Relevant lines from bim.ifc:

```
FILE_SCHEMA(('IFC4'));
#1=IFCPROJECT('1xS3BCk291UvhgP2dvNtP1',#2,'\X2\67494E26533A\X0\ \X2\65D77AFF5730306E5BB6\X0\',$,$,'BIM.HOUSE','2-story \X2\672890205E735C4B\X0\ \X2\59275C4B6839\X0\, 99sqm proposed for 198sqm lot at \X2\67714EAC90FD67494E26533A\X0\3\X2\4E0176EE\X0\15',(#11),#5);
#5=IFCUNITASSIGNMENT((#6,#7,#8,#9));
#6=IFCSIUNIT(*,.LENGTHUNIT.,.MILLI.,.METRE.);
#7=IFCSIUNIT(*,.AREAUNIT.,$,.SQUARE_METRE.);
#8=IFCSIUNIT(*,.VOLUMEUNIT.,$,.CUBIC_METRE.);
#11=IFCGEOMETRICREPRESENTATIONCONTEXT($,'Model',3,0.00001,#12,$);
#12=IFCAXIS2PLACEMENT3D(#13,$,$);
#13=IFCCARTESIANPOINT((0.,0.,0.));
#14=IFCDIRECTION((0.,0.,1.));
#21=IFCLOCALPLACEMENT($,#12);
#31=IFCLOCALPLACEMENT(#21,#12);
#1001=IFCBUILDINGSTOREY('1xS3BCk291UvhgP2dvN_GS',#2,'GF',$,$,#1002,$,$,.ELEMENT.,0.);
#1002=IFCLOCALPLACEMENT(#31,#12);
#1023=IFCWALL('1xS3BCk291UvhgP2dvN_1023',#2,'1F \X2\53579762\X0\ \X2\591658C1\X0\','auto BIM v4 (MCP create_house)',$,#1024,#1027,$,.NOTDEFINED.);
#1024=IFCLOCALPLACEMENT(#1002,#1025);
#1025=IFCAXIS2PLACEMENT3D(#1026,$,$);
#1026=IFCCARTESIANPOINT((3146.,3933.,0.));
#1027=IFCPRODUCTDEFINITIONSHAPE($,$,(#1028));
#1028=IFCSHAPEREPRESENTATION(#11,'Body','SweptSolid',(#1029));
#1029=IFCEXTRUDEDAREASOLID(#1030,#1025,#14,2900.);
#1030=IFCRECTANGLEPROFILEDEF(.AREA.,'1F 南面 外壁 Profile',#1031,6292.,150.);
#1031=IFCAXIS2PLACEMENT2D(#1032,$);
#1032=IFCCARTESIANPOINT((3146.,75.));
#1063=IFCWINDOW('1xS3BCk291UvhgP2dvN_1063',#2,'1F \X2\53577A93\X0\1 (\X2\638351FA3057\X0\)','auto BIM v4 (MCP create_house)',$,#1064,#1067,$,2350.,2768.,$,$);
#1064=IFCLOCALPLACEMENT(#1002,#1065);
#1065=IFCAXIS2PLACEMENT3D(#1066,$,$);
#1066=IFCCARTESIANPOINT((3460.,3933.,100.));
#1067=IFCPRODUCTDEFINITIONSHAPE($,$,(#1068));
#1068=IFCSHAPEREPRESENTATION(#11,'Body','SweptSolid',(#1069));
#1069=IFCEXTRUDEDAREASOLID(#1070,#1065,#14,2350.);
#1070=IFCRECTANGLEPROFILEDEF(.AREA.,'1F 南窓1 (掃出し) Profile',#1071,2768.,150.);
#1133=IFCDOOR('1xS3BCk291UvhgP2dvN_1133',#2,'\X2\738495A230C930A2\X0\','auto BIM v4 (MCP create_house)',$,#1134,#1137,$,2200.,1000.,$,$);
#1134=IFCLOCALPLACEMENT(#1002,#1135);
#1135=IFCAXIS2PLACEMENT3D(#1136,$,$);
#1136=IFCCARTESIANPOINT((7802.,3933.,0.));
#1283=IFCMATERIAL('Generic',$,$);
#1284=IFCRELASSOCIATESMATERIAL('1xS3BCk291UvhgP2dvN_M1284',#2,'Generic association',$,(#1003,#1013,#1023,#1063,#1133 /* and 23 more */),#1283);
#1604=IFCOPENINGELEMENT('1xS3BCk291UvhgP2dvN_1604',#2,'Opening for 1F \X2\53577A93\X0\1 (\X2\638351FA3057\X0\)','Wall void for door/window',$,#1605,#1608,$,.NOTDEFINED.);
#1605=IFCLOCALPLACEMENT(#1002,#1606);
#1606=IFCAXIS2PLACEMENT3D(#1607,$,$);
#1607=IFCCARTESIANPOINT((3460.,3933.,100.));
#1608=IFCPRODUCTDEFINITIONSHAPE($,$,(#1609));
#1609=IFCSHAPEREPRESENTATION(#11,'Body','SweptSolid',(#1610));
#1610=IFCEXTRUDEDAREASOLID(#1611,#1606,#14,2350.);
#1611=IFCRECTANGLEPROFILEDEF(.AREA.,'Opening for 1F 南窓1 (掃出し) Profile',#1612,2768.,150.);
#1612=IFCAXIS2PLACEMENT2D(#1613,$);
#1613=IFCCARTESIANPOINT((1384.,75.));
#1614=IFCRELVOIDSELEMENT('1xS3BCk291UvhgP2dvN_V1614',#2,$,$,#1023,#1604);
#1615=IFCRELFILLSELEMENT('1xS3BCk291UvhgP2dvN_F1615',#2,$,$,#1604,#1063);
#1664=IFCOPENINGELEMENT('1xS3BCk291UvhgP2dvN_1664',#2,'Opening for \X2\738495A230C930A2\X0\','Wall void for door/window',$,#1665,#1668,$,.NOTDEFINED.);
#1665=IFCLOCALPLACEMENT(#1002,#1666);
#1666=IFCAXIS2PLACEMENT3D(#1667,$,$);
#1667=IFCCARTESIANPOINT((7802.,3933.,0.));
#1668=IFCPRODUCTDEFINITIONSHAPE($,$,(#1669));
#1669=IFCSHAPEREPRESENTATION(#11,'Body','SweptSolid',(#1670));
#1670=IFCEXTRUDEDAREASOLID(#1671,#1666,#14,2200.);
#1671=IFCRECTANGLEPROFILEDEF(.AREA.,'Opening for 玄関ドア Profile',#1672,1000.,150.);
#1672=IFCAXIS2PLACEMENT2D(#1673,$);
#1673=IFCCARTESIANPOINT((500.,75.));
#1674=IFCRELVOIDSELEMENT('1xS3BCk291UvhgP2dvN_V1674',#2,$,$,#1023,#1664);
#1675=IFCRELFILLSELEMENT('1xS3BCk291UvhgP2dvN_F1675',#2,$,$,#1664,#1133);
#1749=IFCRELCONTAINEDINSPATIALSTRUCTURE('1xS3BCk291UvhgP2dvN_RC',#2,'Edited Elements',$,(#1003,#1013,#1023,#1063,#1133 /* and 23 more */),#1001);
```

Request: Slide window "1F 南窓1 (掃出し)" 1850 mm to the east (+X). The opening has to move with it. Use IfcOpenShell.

```python
import ifcopenshell
import ifcopenshell.api.geometry
import ifcopenshell.util.placement

model = ifcopenshell.open("bim.ifc")

window = model.by_guid("1xS3BCk291UvhgP2dvN_1063")
opening = window.FillsVoids[0].RelatingOpeningElement
wall = opening.VoidsElements[0].RelatingBuildingElement

wall_matrix = ifcopenshell.util.placement.get_local_placement(wall.ObjectPlacement)
shift = wall_matrix[:3, 0] * 1850.0
before = ifcopenshell.util.placement.get_local_placement(window.ObjectPlacement)[:3, 3].copy()

# The window is not placed relative to its opening, so move both.
for product in (opening, window):
    matrix = ifcopenshell.util.placement.get_local_placement(product.ObjectPlacement)
    matrix[:3, 3] += shift
    ifcopenshell.api.geometry.edit_object_placement(model, product=product, matrix=matrix, is_si=False)

after = ifcopenshell.util.placement.get_local_placement(window.ObjectPlacement)[:3, 3]
print("window moved by", (after - before).round(3) + 0.0)

model.write("bim_rev.ifc")
```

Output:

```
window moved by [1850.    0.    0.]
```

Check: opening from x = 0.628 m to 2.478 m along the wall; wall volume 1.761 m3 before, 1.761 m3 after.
